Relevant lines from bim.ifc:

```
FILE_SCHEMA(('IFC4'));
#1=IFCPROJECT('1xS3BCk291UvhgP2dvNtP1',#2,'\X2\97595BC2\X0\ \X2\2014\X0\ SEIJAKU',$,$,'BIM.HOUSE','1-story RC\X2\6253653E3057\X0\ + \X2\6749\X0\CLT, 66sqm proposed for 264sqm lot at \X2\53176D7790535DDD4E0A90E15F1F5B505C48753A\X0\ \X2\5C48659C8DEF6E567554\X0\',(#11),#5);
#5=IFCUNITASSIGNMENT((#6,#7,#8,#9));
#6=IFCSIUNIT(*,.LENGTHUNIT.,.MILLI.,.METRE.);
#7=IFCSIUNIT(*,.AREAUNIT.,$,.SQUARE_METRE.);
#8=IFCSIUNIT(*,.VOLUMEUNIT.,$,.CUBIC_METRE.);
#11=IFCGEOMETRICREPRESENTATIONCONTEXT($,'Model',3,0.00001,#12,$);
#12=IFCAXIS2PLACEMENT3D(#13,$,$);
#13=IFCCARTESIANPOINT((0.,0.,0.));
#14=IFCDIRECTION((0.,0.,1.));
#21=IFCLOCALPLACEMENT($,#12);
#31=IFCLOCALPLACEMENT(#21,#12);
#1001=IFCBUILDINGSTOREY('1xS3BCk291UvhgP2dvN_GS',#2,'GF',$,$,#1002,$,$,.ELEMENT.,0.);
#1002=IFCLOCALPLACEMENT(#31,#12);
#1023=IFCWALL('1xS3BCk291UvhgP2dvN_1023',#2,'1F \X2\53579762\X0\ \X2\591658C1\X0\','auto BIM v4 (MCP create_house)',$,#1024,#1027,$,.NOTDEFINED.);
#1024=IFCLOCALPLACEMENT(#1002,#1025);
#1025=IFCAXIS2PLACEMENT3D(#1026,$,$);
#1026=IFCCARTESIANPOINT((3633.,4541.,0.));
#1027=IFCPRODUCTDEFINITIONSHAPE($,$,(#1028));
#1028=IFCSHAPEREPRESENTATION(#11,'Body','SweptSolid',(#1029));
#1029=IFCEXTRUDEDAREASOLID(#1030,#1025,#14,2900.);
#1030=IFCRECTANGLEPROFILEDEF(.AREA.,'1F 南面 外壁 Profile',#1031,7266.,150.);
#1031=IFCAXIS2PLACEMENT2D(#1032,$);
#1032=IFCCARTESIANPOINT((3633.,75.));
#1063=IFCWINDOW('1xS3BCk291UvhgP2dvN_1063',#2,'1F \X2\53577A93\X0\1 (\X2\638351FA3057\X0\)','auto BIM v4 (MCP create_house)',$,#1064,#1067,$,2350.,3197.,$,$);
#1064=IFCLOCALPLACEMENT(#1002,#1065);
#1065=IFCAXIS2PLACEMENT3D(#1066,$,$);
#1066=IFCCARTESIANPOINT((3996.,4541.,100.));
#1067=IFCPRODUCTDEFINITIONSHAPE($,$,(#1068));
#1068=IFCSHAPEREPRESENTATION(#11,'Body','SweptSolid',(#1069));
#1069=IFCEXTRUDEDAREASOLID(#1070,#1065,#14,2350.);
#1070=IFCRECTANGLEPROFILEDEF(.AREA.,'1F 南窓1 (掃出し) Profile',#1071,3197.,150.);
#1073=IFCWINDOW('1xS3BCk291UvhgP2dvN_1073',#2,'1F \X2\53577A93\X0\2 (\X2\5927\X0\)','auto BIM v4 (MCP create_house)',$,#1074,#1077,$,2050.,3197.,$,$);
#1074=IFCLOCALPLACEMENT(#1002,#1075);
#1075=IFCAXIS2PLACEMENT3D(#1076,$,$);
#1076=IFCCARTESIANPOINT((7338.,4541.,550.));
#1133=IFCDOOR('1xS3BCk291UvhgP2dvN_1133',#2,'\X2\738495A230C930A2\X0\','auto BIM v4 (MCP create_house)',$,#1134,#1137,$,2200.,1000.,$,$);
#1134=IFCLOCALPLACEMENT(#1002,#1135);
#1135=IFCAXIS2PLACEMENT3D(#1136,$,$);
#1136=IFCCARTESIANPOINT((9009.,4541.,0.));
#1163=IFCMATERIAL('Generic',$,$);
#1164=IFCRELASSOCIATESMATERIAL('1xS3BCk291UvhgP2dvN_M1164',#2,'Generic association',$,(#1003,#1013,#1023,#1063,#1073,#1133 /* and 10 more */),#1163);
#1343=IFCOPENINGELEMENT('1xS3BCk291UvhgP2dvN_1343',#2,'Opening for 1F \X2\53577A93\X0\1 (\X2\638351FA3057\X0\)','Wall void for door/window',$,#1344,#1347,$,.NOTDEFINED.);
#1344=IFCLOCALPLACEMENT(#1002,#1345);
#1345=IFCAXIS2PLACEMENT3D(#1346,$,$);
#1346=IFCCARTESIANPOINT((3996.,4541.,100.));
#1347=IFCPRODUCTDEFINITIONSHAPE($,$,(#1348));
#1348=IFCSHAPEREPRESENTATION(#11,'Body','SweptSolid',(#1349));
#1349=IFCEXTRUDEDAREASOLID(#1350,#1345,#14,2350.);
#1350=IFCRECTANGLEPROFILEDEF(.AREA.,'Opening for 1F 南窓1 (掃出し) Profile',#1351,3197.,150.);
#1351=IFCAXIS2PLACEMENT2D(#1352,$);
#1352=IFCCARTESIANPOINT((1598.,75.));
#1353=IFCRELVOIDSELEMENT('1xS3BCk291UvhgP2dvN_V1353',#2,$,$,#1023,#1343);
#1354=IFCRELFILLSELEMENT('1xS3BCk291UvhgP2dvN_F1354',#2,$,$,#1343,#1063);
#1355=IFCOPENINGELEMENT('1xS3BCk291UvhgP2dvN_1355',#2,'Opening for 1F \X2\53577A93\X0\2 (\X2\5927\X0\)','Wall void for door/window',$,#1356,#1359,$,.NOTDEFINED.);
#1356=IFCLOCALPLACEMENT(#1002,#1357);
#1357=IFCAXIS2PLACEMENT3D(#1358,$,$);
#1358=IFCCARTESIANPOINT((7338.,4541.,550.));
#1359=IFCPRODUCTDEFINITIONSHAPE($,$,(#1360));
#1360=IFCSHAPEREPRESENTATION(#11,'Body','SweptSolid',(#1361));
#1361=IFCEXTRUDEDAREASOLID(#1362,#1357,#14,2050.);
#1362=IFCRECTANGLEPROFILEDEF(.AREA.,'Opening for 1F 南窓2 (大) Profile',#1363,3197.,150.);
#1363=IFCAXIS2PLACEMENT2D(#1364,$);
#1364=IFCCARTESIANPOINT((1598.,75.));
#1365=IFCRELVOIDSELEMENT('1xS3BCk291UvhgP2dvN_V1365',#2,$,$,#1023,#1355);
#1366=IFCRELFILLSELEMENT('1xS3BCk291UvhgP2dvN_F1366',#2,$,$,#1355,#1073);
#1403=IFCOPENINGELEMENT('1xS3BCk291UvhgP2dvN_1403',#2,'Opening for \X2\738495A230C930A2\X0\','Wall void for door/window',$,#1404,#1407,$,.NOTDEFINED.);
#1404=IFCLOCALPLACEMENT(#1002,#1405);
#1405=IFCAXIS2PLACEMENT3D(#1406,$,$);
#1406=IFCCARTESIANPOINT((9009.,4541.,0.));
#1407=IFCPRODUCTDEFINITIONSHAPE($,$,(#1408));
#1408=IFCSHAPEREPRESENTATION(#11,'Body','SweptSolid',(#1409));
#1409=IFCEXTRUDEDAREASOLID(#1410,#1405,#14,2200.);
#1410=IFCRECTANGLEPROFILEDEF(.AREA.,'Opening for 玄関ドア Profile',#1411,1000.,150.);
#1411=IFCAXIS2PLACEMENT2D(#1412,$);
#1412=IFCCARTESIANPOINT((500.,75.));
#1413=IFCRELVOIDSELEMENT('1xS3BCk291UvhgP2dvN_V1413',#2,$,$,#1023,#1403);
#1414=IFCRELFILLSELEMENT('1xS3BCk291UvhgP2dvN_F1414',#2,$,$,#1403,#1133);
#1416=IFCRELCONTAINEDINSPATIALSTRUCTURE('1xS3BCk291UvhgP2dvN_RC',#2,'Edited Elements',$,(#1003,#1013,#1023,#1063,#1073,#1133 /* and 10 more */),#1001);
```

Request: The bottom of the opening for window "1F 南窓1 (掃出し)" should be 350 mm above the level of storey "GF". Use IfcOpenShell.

```python
import numpy as np
import ifcopenshell
import ifcopenshell.api.geometry
import ifcopenshell.geom
import ifcopenshell.util.element
import ifcopenshell.util.placement
import ifcopenshell.util.shape
import ifcopenshell.util.unit

model = ifcopenshell.open("bim.ifc")
unit_scale = ifcopenshell.util.unit.calculate_unit_scale(model)

window = model.by_guid("1xS3BCk291UvhgP2dvN_1063")
opening = window.FillsVoids[0].RelatingOpeningElement
storey = ifcopenshell.util.element.get_container(window, ifc_class="IfcBuildingStorey")
level = ifcopenshell.util.placement.get_local_placement(storey.ObjectPlacement)[2, 3]

# The opening's origin need not be at the sill, so measure its lowest point.
shape = ifcopenshell.geom.create_shape(ifcopenshell.geom.settings(), opening)
bottom = ifcopenshell.util.shape.get_shape_bottom_elevation(shape, shape.geometry) / unit_scale
dz = level + 0.35 / unit_scale - bottom

shift = np.array([0.0, 0.0, dz])
# The window is not placed relative to its opening, so move both.
for product in (opening, window):
    matrix = ifcopenshell.util.placement.get_local_placement(product.ObjectPlacement)
    matrix[:3, 3] += shift
    ifcopenshell.api.geometry.edit_object_placement(model, product=product, matrix=matrix, is_si=False)

print(f"moved by {dz * unit_scale:+.3f} m")

model.write("bim_rev.ifc")
```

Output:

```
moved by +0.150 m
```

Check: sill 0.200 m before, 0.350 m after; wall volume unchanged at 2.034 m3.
